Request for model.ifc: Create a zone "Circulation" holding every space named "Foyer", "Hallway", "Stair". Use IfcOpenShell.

First a look at what the model holds.

```python
import ifcopenshell

model = ifcopenshell.open("model.ifc")
print(model.schema)
seen = {}
for space in model.by_type("IfcSpace"):
    seen[space.LongName] = seen.get(space.LongName, 0) + 1
for name, count in sorted(seen.items(), key=str):
    print(count, "x", name)
print("zones:", [z.Name for z in model.by_type("IfcZone")][:20])
```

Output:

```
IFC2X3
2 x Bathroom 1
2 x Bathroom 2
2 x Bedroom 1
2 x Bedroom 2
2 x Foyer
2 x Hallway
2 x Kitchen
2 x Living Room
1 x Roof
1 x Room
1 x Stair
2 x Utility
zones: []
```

```python
import ifcopenshell
import ifcopenshell.api.group
import ifcopenshell.api.root

model = ifcopenshell.open("model.ifc")

names = {"Foyer", "Hallway", "Stair"}
spaces = [s for s in model.by_type("IfcSpace") if s.LongName in names]

zone = ifcopenshell.api.root.create_entity(model, ifc_class="IfcZone", name="Circulation")
ifcopenshell.api.group.assign_group(model, products=spaces, group=zone)
print(len(spaces), "spaces in", zone.Name)

model.write("model_v2.ifc")
```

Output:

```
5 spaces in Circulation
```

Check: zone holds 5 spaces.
